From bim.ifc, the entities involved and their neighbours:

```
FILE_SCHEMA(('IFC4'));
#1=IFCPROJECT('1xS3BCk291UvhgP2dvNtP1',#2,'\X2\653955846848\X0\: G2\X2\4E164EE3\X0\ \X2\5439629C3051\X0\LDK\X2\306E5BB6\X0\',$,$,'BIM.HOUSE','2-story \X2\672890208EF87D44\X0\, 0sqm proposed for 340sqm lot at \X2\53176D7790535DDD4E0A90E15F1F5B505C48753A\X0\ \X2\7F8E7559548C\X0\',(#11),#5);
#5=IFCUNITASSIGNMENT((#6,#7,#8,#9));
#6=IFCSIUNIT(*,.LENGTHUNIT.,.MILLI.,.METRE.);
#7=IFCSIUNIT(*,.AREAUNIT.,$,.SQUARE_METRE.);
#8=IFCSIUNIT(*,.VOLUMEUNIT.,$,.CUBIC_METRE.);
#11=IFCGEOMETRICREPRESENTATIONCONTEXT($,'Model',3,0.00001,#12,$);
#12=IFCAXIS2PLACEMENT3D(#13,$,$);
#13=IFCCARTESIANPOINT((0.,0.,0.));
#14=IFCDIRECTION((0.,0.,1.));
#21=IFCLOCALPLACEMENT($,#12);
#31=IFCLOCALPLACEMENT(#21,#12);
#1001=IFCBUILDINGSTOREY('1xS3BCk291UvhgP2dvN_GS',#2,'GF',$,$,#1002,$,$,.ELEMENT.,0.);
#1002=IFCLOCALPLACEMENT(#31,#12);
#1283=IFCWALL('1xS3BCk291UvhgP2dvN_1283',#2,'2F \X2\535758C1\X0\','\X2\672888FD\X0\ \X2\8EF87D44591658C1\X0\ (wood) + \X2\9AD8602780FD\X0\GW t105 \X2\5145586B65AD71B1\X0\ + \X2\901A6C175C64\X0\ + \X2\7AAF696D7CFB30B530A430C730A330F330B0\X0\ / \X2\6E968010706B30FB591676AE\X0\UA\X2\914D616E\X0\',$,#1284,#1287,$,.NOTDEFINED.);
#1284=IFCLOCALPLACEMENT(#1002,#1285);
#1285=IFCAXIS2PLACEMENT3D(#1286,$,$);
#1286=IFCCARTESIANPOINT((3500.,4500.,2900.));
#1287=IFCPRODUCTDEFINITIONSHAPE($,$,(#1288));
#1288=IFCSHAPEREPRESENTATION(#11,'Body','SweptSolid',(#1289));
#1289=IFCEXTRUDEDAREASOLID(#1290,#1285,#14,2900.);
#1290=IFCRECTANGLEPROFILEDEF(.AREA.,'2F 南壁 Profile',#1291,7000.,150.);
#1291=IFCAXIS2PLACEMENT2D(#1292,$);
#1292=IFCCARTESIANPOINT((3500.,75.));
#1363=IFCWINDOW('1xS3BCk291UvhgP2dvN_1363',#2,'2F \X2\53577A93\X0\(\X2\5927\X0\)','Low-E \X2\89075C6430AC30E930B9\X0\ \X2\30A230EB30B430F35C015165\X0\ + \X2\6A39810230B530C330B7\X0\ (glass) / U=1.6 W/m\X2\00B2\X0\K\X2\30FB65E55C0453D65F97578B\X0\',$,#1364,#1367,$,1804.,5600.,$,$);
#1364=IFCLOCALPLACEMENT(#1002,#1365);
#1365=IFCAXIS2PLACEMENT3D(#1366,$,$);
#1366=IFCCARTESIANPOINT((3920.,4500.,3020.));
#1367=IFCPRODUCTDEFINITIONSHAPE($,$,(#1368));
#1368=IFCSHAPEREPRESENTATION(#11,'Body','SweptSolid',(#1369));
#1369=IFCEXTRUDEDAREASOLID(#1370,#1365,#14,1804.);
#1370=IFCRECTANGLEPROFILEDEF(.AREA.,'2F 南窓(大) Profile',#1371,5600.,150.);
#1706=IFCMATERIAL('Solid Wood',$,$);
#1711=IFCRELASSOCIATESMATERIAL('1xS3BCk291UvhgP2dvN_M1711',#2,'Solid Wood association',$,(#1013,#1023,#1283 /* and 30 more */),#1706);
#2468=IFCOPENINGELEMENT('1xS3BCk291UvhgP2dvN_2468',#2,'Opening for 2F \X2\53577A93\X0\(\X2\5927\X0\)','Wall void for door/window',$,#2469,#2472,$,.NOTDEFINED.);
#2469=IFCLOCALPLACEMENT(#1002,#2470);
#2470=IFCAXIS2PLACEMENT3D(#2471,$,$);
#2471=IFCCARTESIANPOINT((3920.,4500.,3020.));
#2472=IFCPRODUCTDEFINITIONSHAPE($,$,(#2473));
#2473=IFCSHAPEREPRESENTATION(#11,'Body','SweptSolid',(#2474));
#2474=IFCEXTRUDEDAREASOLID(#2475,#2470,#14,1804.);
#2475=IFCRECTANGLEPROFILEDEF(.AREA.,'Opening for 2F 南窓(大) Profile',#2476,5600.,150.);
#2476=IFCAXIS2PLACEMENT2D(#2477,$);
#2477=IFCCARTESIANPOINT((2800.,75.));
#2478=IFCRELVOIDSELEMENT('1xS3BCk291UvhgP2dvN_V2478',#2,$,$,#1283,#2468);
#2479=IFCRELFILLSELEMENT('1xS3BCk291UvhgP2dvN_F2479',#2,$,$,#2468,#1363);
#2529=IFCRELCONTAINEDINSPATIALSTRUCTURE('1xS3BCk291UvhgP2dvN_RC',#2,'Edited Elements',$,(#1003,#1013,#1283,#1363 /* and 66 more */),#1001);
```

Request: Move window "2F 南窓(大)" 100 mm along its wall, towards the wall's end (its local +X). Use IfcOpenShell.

```python
import ifcopenshell
import ifcopenshell.api.geometry
import ifcopenshell.util.placement

model = ifcopenshell.open("bim.ifc")

window = model.by_id(1363)
opening = window.FillsVoids[0].RelatingOpeningElement
wall = opening.VoidsElements[0].RelatingBuildingElement

wall_matrix = ifcopenshell.util.placement.get_local_placement(wall.ObjectPlacement)
shift = wall_matrix[:3, 0] * 100.0
before = ifcopenshell.util.placement.get_local_placement(window.ObjectPlacement)[:3, 3].copy()

# The window is not placed relative to its opening, so move both.
for product in (opening, window):
    matrix = ifcopenshell.util.placement.get_local_placement(product.ObjectPlacement)
    matrix[:3, 3] += shift
    ifcopenshell.api.geometry.edit_object_placement(model, product=product, matrix=matrix, is_si=False)

after = ifcopenshell.util.placement.get_local_placement(window.ObjectPlacement)[:3, 3]
print("window moved by", (after - before).round(3) + 0.0)

model.write("bim_v2.ifc")
```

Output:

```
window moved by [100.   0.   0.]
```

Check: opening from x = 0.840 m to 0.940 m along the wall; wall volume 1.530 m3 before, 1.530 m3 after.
